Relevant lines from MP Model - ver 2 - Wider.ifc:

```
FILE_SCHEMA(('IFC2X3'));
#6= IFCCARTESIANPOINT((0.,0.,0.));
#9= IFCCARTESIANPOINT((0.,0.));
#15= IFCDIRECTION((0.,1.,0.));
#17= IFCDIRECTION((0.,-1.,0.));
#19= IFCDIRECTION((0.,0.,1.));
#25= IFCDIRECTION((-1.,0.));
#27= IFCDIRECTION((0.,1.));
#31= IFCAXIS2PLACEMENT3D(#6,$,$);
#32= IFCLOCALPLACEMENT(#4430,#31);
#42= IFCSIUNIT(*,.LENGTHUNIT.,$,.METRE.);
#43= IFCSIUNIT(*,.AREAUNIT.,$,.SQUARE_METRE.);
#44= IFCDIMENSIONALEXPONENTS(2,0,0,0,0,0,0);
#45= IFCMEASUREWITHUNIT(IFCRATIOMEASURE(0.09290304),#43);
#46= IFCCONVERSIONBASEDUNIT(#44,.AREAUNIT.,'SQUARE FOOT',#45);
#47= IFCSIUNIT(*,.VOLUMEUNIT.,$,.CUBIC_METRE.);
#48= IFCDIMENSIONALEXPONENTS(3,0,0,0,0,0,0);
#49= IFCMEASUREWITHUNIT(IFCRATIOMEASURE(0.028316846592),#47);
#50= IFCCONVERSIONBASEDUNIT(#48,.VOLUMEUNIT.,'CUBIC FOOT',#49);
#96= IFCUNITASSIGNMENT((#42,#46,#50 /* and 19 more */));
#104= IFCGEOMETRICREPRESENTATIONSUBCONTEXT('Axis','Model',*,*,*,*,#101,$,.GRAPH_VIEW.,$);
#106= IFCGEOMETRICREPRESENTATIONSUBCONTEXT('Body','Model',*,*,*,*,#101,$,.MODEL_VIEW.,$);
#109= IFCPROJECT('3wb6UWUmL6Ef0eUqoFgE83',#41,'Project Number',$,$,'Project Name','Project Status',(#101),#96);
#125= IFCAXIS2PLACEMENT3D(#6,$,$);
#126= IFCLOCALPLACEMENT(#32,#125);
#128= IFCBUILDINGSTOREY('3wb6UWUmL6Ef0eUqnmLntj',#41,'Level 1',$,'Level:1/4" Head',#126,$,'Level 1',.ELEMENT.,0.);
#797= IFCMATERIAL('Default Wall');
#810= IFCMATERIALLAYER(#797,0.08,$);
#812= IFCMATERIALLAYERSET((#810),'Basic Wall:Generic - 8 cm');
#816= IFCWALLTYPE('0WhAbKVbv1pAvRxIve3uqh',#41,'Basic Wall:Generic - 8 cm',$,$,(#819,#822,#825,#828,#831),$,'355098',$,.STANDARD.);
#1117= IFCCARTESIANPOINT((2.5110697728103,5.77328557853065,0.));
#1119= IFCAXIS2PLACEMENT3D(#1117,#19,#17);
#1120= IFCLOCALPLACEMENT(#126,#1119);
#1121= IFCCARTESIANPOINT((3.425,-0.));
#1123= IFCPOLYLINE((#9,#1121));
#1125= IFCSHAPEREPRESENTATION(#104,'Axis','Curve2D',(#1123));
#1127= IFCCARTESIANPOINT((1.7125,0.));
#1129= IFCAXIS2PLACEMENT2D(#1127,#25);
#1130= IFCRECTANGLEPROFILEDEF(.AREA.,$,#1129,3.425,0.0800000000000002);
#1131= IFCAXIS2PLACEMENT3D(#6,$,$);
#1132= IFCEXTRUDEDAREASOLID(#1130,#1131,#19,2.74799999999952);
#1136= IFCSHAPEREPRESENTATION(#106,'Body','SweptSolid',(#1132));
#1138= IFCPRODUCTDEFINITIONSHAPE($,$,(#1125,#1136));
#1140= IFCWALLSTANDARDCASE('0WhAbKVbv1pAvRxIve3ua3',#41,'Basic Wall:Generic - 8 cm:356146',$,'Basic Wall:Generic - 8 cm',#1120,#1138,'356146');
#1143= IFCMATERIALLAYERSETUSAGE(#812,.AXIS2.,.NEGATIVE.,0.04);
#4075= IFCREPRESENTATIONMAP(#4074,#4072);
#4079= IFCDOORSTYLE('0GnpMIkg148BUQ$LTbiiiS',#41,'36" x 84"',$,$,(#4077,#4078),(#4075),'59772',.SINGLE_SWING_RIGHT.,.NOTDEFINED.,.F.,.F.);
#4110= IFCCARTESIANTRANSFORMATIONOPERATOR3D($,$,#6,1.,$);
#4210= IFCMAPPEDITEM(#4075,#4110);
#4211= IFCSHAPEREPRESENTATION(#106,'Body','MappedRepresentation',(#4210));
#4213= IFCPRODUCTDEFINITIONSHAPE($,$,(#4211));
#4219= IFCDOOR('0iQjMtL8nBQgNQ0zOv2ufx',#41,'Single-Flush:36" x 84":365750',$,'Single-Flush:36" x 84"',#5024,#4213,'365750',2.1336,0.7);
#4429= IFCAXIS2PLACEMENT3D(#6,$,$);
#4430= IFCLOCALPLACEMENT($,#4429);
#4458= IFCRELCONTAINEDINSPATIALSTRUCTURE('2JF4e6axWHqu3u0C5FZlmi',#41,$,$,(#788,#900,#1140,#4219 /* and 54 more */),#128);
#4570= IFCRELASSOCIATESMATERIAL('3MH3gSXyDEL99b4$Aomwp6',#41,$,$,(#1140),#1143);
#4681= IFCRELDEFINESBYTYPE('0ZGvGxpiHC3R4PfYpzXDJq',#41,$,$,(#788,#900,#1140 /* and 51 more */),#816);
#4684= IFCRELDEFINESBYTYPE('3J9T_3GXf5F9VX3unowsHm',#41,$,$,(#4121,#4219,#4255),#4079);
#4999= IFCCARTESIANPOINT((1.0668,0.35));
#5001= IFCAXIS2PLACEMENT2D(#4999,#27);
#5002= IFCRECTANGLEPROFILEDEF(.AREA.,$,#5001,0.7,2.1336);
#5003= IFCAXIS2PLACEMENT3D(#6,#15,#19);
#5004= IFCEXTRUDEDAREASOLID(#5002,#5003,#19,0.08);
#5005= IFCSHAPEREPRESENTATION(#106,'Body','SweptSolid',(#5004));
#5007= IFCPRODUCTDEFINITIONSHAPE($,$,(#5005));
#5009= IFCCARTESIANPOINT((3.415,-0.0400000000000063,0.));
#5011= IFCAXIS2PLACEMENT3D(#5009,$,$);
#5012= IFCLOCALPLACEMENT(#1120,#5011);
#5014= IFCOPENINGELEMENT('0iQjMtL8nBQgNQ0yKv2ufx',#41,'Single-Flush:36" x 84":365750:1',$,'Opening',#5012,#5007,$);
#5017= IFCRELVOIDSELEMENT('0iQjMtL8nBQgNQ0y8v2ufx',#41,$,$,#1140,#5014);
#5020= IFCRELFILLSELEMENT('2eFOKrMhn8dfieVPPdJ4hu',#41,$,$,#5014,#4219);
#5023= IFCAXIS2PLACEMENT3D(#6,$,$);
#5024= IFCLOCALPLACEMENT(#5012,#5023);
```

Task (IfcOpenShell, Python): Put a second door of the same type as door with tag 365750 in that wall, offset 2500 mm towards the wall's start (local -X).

```python
import ifcopenshell
import ifcopenshell.api.feature
import ifcopenshell.api.geometry
import ifcopenshell.api.root
import ifcopenshell.geom
import ifcopenshell.util.element
import ifcopenshell.util.placement
import ifcopenshell.util.shape
import ifcopenshell.util.unit

model = ifcopenshell.open("MP Model - ver 2 - Wider.ifc")
unit_scale = ifcopenshell.util.unit.calculate_unit_scale(model)
settings = ifcopenshell.geom.settings()


def volume(element):
    """Net volume in cubic metres, openings subtracted."""
    shape = ifcopenshell.geom.create_shape(settings, element)
    return ifcopenshell.util.shape.get_volume(shape.geometry)


def reuse_history(source, copy):
    """copy_class also copies each property set's owner history, people and application; keep the originals."""
    for rel in copy.IsDefinedBy:
        if rel.is_a("IfcRelDefinesByProperties") and (history := rel.RelatingPropertyDefinition.OwnerHistory):
            rel.RelatingPropertyDefinition.OwnerHistory = source.OwnerHistory
            ifcopenshell.util.element.remove_deep2(model, history)


door = model.by_guid("0iQjMtL8nBQgNQ0zOv2ufx")
opening = door.FillsVoids[0].RelatingOpeningElement
wall = opening.VoidsElements[0].RelatingBuildingElement
before = volume(wall)
shift = ifcopenshell.util.placement.get_local_placement(wall.ObjectPlacement)[:3, 0] * -2.5 / unit_scale

# copy_class copies the void relationship, type, container and properties, but no geometry.
new_opening = ifcopenshell.api.root.copy_class(model, product=opening)
new_opening.Representation = ifcopenshell.util.element.copy_deep(
    model, opening.Representation, exclude=["IfcGeometricRepresentationContext", "IfcRepresentationMap"]
)
new_opening.Name = 'Single-Flush:36" x 84"'
new_door = ifcopenshell.api.root.copy_class(model, product=door)
new_door.Representation = ifcopenshell.util.element.copy_deep(
    model, door.Representation, exclude=["IfcGeometricRepresentationContext", "IfcRepresentationMap"]
)
new_door.Name = 'Single-Flush:36" x 84"'
new_door.Tag = None
reuse_history(door, new_door)
fills = ifcopenshell.api.feature.add_filling(model, opening=new_opening, element=new_door)
fills.OwnerHistory = new_door.OwnerHistory  # required in IFC2X3

for old, new in ((opening, new_opening), (door, new_door)):
    matrix = ifcopenshell.util.placement.get_local_placement(old.ObjectPlacement)
    matrix[:3, 3] += shift
    ifcopenshell.api.geometry.edit_object_placement(model, product=new, matrix=matrix, is_si=False)

after = volume(wall)

print(f"wall volume {before:.3f} -> {after:.3f} m3")

model.write("MP Model - ver 2 - Wider-out.ifc")
```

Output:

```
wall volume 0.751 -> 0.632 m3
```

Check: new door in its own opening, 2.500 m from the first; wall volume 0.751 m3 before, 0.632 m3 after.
